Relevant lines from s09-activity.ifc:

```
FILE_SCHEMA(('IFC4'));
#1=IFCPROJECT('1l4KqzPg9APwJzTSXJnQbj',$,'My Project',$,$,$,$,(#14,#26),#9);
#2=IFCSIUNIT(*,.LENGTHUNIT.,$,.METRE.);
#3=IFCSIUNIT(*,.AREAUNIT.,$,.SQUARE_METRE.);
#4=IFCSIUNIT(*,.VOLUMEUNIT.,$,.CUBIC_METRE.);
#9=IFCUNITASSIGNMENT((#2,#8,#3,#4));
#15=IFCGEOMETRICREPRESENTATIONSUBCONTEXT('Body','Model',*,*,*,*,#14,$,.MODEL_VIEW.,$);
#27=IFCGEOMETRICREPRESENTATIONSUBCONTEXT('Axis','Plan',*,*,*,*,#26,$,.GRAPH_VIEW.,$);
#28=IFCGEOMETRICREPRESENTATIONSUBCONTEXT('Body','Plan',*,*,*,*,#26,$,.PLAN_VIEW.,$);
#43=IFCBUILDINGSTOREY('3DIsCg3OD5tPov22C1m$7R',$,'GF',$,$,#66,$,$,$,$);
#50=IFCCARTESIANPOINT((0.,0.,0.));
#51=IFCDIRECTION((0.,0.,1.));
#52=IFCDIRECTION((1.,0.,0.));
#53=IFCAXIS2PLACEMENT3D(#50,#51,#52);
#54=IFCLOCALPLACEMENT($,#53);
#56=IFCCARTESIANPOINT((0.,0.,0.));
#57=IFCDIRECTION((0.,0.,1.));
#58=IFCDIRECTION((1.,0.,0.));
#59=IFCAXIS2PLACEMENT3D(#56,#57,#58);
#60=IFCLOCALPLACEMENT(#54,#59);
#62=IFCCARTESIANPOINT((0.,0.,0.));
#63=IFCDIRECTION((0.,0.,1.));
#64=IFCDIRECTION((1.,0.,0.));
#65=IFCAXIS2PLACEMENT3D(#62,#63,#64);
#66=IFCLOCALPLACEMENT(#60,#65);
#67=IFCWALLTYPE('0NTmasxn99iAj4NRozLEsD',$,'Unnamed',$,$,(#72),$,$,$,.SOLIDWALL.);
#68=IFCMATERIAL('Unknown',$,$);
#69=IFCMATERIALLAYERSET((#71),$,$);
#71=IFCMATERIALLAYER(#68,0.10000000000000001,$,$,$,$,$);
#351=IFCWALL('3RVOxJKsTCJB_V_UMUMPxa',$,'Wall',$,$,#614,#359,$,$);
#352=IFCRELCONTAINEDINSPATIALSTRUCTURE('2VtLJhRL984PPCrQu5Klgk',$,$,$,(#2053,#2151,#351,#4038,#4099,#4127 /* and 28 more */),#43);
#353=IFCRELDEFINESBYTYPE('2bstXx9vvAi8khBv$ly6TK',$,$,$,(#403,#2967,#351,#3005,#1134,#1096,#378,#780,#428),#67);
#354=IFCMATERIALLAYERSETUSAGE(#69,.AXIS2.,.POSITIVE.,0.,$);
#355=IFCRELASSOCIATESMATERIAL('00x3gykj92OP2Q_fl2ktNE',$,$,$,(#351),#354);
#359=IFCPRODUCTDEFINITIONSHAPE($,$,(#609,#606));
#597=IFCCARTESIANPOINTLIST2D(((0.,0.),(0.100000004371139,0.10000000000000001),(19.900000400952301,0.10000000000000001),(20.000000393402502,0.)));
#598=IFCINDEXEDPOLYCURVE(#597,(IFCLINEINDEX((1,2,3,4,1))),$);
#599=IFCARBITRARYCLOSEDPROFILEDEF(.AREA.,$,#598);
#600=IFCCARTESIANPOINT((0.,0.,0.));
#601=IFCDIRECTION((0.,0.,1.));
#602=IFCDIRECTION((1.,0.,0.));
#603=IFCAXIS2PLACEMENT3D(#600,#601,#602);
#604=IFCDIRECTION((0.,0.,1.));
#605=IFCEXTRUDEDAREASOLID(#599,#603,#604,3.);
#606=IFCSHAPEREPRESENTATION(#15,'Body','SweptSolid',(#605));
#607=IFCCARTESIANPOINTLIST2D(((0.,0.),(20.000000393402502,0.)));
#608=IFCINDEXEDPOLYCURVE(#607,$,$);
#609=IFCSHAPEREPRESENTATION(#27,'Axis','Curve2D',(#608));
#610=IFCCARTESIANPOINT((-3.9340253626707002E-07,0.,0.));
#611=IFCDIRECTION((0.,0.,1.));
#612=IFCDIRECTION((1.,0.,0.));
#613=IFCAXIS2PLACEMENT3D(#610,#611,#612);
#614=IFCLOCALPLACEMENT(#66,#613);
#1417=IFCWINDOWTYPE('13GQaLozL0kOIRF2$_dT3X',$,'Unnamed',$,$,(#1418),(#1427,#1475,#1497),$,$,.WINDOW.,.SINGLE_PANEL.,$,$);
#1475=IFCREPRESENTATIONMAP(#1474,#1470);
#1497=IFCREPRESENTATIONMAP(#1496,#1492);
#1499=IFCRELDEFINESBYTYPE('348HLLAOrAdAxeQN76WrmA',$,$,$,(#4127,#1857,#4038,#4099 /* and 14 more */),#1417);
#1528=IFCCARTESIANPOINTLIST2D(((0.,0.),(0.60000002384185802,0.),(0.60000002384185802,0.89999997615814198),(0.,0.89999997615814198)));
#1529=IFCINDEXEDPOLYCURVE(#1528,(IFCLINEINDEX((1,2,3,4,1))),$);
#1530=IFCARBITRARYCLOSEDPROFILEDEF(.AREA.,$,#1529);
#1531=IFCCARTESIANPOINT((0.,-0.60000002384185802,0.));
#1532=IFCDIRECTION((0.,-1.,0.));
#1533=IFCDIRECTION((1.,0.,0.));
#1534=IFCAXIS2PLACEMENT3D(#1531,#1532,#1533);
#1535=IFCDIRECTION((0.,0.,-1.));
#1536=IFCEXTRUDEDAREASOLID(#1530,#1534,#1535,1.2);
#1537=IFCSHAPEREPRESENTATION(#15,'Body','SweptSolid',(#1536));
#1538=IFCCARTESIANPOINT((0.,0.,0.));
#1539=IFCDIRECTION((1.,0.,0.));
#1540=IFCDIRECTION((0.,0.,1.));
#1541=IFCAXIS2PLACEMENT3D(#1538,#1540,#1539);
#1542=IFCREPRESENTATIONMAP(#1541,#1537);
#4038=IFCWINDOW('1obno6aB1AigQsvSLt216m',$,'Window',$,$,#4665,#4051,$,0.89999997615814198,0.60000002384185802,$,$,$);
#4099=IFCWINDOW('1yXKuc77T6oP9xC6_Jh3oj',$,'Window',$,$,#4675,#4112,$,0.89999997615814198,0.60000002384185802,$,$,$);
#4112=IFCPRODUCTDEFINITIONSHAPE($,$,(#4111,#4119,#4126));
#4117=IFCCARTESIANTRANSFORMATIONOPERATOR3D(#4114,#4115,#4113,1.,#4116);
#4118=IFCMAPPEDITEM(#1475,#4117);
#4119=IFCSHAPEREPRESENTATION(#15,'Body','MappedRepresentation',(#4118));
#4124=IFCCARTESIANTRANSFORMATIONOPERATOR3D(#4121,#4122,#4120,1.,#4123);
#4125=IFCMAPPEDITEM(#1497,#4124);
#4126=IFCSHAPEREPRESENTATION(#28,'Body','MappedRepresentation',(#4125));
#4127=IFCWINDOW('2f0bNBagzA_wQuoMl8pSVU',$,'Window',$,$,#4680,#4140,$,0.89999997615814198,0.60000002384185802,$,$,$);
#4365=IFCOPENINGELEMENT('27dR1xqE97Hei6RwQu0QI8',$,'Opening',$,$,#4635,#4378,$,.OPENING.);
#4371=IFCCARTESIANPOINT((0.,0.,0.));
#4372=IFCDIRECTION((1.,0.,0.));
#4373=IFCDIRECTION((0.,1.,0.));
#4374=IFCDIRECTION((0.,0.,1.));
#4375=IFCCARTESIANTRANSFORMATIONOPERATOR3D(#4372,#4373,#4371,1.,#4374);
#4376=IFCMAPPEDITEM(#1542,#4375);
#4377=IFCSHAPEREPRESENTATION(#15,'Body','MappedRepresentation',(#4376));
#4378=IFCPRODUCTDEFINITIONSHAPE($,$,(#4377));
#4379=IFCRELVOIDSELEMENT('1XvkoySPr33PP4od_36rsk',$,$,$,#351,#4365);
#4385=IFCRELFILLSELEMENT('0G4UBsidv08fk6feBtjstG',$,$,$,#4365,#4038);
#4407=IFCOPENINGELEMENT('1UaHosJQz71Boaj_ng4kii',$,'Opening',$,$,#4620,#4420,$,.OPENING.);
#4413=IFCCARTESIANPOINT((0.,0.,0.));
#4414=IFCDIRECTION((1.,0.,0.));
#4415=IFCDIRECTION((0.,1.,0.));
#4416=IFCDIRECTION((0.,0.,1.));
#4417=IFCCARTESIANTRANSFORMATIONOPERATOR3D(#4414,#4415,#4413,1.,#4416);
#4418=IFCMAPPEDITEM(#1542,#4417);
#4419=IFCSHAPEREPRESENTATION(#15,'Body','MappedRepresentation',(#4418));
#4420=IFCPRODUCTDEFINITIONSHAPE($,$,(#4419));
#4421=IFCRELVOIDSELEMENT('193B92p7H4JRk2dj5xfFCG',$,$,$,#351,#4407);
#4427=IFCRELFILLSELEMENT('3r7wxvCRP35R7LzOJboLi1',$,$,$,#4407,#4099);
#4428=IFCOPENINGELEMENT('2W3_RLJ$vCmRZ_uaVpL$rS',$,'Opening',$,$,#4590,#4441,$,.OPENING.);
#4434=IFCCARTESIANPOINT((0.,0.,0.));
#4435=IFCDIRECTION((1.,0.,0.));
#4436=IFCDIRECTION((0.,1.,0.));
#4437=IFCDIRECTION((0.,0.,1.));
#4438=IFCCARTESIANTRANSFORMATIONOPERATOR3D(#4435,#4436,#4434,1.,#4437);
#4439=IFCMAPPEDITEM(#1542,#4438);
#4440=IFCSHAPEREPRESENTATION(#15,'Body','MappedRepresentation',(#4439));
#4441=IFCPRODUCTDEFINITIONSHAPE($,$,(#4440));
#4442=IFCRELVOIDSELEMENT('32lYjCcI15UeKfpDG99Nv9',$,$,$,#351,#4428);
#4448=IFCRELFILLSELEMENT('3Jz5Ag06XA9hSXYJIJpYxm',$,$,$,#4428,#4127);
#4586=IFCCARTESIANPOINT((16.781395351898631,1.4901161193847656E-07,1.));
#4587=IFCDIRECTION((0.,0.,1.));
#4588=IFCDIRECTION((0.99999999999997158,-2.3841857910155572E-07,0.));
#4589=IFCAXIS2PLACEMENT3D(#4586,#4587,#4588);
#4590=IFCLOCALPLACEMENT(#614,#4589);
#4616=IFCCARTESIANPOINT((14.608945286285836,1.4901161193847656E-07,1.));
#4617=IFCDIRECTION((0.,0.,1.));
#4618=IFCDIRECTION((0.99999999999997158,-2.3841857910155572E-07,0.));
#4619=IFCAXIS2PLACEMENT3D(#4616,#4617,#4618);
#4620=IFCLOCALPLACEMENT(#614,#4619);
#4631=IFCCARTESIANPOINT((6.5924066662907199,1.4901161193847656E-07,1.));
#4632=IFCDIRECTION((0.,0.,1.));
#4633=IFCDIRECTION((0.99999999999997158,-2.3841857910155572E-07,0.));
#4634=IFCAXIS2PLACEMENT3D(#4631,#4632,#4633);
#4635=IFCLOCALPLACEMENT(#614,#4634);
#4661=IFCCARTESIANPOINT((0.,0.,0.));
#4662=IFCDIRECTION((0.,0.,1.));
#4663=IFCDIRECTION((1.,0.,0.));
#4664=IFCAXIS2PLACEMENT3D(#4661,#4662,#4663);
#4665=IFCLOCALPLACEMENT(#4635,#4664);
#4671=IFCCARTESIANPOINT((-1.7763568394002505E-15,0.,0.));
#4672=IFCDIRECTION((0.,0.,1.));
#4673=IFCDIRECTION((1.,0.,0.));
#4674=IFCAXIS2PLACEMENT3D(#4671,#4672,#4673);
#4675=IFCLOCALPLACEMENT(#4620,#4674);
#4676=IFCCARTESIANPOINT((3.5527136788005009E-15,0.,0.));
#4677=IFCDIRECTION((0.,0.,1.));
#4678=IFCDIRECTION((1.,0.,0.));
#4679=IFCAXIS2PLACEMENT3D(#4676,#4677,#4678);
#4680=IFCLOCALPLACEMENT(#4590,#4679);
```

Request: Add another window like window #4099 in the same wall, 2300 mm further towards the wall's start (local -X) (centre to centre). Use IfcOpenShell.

```python
import ifcopenshell
import ifcopenshell.api.feature
import ifcopenshell.api.geometry
import ifcopenshell.api.root
import ifcopenshell.geom
import ifcopenshell.util.element
import ifcopenshell.util.placement
import ifcopenshell.util.shape

model = ifcopenshell.open("s09-activity.ifc")
settings = ifcopenshell.geom.settings()


def volume(element):
    """Net volume in cubic metres, openings subtracted."""
    shape = ifcopenshell.geom.create_shape(settings, element)
    return ifcopenshell.util.shape.get_volume(shape.geometry)


window = model.by_guid("1yXKuc77T6oP9xC6_Jh3oj")
opening = window.FillsVoids[0].RelatingOpeningElement
wall = opening.VoidsElements[0].RelatingBuildingElement
before = volume(wall)
shift = ifcopenshell.util.placement.get_local_placement(wall.ObjectPlacement)[:3, 0] * -2.3

# copy_class copies the void relationship, type, container and properties, but no geometry.
new_opening = ifcopenshell.api.root.copy_class(model, product=opening)
new_opening.Representation = ifcopenshell.util.element.copy_deep(
    model, opening.Representation, exclude=["IfcGeometricRepresentationContext", "IfcRepresentationMap"]
)
new_window = ifcopenshell.api.root.copy_class(model, product=window)
new_window.Representation = ifcopenshell.util.element.copy_deep(
    model, window.Representation, exclude=["IfcGeometricRepresentationContext", "IfcRepresentationMap"]
)
ifcopenshell.api.feature.add_filling(model, opening=new_opening, element=new_window)

for old, new in ((opening, new_opening), (window, new_window)):
    matrix = ifcopenshell.util.placement.get_local_placement(old.ObjectPlacement)
    matrix[:3, 3] += shift
    ifcopenshell.api.geometry.edit_object_placement(model, product=new, matrix=matrix, is_si=False)

after = volume(wall)

print(f"wall volume {before:.3f} -> {after:.3f} m3")

model.write("s09-activity_updated.ifc")
```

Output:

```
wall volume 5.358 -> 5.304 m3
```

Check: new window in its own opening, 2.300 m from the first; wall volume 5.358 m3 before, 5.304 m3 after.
